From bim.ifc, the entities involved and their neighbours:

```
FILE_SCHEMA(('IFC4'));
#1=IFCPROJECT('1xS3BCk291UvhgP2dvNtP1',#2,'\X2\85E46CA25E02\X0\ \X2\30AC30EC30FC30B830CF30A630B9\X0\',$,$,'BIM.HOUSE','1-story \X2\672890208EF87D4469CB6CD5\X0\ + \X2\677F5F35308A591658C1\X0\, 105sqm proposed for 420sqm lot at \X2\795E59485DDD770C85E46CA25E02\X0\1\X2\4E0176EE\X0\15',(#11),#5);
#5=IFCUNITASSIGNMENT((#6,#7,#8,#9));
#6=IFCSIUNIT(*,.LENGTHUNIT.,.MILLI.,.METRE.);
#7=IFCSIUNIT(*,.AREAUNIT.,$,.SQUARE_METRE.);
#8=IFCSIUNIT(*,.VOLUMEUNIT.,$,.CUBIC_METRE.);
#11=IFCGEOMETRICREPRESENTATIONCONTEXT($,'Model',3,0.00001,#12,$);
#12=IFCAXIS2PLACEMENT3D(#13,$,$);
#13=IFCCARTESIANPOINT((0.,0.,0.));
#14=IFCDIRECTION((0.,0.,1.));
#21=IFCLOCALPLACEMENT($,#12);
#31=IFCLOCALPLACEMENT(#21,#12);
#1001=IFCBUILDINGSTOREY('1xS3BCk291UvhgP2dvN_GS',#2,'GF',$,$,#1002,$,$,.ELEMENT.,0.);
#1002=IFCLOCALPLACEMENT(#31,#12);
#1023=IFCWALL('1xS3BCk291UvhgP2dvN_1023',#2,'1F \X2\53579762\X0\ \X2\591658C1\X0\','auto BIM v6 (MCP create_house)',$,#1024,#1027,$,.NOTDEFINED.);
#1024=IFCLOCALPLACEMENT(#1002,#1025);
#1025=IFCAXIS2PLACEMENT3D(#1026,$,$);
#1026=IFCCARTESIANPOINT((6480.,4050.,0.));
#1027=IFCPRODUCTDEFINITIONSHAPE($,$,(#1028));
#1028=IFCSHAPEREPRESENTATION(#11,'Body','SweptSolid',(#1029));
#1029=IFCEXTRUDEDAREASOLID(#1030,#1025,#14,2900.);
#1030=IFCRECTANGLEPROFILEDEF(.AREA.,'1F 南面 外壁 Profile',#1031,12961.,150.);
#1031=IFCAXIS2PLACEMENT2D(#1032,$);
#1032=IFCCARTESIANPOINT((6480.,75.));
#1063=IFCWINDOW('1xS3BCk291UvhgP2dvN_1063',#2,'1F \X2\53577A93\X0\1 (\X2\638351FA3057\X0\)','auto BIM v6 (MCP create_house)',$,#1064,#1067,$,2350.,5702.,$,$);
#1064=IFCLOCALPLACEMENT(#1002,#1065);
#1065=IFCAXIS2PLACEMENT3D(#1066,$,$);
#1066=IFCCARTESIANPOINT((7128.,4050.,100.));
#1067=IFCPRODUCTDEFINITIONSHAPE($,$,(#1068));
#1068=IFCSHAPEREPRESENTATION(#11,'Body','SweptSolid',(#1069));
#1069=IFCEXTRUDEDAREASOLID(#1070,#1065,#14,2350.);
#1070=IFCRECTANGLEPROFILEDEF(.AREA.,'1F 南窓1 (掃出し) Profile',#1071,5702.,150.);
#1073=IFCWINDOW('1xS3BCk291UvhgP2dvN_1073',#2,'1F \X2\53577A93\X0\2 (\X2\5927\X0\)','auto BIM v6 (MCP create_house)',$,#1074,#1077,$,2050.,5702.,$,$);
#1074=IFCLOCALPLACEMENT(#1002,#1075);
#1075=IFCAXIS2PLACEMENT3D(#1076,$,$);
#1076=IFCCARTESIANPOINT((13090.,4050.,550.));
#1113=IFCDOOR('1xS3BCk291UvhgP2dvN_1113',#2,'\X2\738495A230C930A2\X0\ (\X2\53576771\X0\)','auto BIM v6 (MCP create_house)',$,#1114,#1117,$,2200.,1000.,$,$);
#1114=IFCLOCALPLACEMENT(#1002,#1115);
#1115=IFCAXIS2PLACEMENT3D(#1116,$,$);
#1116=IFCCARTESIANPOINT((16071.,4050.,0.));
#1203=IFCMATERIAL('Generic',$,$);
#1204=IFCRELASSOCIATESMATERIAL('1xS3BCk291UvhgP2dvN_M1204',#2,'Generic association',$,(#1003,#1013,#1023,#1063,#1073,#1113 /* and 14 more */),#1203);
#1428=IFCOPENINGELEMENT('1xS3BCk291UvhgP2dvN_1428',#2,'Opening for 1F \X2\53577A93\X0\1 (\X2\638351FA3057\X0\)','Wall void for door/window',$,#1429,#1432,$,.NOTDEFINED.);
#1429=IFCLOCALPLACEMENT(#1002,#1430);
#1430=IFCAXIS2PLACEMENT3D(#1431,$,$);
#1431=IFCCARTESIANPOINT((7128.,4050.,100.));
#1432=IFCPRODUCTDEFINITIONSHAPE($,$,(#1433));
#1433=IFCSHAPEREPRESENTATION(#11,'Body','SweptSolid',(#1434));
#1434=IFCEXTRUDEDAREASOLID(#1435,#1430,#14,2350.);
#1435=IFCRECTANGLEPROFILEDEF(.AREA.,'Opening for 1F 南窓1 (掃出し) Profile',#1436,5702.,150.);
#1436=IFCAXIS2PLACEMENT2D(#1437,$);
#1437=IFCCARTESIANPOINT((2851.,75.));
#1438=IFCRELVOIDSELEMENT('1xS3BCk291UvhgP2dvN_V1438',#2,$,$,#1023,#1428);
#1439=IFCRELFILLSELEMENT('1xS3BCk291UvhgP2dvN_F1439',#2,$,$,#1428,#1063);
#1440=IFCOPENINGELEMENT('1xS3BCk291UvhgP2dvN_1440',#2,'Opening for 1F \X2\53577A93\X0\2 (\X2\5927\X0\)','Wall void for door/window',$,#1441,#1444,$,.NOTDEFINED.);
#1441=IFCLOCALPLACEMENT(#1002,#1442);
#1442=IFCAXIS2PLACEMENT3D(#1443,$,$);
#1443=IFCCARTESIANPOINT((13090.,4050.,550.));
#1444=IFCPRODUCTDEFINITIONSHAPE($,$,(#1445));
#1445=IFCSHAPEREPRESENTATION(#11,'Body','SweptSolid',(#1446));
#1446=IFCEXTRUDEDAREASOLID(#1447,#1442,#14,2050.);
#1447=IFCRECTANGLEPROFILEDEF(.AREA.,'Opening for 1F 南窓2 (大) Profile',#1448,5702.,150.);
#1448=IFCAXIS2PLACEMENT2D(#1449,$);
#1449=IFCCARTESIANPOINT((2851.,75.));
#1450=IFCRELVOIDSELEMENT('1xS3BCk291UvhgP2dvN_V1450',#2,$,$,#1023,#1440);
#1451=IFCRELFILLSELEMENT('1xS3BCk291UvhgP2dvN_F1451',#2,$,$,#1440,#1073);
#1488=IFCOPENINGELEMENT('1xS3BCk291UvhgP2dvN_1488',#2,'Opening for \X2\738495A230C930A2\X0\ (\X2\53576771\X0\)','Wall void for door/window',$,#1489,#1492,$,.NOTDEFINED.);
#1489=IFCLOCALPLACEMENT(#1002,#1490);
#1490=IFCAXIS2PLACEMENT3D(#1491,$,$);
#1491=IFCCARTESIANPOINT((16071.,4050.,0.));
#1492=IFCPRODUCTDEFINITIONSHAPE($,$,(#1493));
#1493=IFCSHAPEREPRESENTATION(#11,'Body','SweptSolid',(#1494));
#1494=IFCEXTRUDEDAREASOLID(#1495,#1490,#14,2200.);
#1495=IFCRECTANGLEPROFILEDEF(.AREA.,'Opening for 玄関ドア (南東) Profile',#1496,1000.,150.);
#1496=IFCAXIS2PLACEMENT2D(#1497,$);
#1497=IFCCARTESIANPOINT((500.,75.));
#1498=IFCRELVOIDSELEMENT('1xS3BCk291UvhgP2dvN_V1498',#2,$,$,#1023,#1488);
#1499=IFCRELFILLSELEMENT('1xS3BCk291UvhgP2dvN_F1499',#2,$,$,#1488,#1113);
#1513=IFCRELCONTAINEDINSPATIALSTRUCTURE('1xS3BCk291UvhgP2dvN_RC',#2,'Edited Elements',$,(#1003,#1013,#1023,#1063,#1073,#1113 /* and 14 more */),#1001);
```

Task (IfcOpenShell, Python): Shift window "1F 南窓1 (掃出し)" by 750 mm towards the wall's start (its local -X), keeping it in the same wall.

```python
import ifcopenshell
import ifcopenshell.api.geometry
import ifcopenshell.util.placement
import ifcopenshell.util.unit

model = ifcopenshell.open("bim.ifc")
unit_scale = ifcopenshell.util.unit.calculate_unit_scale(model)

window = model.by_id(1063)
opening = window.FillsVoids[0].RelatingOpeningElement
wall = opening.VoidsElements[0].RelatingBuildingElement

wall_matrix = ifcopenshell.util.placement.get_local_placement(wall.ObjectPlacement)
shift = wall_matrix[:3, 0] * -0.75 / unit_scale
before = ifcopenshell.util.placement.get_local_placement(window.ObjectPlacement)[:3, 3].copy()

# The window is not placed relative to its opening, so move both.
for product in (opening, window):
    matrix = ifcopenshell.util.placement.get_local_placement(product.ObjectPlacement)
    matrix[:3, 3] += shift
    ifcopenshell.api.geometry.edit_object_placement(model, product=product, matrix=matrix, is_si=False)

after = ifcopenshell.util.placement.get_local_placement(window.ObjectPlacement)[:3, 3]
print("window moved by", (after - before).round(3) + 0.0)

model.write("bim-out.ifc")
```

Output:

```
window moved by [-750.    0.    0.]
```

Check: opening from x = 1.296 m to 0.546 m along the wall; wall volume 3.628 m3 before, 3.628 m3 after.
